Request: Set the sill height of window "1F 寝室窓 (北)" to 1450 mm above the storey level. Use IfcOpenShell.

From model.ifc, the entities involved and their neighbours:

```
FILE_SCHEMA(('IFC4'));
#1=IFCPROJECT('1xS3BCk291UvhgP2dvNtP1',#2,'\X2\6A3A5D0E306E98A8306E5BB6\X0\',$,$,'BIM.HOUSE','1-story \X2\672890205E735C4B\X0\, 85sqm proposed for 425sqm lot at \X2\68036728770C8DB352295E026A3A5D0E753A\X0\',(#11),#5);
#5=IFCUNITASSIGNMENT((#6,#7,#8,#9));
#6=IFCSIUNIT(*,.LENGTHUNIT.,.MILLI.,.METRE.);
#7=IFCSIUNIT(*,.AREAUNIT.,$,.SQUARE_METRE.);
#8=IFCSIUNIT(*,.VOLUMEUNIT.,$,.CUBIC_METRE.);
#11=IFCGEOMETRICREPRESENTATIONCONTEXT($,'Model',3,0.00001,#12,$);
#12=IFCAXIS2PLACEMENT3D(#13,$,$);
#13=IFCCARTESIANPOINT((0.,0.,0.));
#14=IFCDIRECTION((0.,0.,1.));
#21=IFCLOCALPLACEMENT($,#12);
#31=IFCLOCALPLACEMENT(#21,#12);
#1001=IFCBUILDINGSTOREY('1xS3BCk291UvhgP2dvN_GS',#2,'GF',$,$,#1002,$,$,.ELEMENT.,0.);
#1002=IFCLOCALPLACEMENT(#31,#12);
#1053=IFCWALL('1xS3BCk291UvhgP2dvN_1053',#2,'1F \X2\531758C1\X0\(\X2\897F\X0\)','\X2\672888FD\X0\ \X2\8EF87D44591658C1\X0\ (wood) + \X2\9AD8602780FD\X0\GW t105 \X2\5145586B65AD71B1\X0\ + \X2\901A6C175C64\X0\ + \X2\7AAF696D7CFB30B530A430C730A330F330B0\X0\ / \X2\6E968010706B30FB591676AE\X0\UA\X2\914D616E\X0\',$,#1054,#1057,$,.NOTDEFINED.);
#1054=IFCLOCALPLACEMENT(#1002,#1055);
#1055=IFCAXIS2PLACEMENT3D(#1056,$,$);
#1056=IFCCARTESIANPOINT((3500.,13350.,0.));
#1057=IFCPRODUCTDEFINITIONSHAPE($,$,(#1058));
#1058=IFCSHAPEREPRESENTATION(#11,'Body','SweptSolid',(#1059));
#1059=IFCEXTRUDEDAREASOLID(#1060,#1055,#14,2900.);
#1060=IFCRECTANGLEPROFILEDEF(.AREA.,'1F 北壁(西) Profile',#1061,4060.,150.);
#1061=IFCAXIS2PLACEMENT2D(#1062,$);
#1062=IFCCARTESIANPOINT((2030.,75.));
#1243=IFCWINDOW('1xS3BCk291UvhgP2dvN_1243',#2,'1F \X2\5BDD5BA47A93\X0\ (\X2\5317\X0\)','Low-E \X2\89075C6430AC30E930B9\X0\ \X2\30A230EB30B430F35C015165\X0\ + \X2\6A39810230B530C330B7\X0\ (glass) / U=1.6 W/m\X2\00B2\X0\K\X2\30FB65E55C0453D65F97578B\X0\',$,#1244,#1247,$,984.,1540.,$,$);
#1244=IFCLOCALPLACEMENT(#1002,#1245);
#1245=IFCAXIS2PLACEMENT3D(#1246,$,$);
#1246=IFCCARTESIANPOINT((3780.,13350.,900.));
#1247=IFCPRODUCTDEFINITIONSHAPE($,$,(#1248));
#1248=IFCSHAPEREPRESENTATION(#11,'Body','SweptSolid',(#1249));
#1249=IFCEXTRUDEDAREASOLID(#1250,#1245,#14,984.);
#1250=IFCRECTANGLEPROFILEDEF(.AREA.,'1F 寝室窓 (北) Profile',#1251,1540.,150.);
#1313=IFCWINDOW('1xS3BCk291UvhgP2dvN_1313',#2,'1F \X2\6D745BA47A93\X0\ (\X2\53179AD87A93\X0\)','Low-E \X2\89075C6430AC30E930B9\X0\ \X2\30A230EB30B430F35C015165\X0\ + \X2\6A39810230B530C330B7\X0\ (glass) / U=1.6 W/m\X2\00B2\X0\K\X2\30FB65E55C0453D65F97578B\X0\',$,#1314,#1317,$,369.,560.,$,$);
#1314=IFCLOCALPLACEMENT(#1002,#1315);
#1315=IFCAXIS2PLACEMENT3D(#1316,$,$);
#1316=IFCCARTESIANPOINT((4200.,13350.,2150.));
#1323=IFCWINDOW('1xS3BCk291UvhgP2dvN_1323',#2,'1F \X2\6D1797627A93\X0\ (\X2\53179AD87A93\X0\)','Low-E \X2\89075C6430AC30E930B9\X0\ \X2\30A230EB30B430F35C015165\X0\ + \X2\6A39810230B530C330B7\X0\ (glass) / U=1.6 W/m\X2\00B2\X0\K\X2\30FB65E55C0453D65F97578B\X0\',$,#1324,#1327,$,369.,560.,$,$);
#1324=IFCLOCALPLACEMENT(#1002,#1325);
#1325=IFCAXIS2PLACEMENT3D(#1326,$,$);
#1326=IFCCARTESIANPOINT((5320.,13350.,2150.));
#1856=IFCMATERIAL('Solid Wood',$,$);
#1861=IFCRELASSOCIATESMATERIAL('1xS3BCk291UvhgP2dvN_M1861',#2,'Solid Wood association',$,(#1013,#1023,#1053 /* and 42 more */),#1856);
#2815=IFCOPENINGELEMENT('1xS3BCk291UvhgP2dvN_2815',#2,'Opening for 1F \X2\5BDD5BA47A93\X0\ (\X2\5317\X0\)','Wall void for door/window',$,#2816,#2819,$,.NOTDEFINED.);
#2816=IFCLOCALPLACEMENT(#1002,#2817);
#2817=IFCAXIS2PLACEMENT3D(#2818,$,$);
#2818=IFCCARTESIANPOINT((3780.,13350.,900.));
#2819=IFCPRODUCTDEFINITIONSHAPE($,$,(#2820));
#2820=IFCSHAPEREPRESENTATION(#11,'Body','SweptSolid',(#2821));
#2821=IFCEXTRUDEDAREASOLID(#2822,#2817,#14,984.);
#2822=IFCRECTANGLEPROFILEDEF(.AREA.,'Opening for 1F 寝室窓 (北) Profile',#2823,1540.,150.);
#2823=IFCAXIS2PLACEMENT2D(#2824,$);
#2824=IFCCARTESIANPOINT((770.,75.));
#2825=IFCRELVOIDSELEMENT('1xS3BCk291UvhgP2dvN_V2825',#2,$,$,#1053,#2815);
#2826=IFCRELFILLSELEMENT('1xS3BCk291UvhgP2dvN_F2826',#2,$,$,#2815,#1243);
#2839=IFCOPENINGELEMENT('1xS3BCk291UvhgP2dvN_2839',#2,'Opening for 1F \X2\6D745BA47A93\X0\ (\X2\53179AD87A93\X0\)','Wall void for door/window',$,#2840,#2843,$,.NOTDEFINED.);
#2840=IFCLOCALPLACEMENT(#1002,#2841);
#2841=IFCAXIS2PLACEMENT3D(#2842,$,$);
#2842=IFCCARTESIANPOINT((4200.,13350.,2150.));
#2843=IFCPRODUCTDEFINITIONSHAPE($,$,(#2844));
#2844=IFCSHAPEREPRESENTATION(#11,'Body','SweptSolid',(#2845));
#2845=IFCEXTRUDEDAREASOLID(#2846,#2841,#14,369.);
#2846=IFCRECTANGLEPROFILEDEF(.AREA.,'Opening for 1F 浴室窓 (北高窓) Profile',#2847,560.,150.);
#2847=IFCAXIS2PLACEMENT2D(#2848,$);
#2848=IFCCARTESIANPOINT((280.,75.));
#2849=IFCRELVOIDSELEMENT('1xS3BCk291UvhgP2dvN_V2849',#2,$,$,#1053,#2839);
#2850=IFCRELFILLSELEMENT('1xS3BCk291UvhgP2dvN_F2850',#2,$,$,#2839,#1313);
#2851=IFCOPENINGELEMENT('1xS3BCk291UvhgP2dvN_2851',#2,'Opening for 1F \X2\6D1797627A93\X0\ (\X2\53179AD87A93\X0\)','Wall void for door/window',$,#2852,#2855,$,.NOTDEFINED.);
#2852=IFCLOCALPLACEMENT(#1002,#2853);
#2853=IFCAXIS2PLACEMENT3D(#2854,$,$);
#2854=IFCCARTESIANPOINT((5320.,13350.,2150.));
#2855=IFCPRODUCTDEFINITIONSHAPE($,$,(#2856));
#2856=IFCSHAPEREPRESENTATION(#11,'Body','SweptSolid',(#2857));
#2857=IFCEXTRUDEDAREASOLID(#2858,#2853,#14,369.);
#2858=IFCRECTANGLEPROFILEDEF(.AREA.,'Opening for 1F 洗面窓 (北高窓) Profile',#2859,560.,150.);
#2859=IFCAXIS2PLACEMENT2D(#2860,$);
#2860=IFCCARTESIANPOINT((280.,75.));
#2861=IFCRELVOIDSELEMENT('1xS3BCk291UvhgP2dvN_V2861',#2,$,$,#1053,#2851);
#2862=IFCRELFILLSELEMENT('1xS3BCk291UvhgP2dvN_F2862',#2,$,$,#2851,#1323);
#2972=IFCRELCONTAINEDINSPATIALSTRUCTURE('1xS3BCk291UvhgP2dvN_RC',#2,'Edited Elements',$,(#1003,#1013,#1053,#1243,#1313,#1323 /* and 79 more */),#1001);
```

```python
import numpy as np
import ifcopenshell
import ifcopenshell.api.geometry
import ifcopenshell.geom
import ifcopenshell.util.element
import ifcopenshell.util.placement
import ifcopenshell.util.shape
import ifcopenshell.util.unit

model = ifcopenshell.open("model.ifc")
unit_scale = ifcopenshell.util.unit.calculate_unit_scale(model)

window = model.by_guid("1xS3BCk291UvhgP2dvN_1243")
opening = window.FillsVoids[0].RelatingOpeningElement
storey = ifcopenshell.util.element.get_container(window, ifc_class="IfcBuildingStorey")
level = ifcopenshell.util.placement.get_local_placement(storey.ObjectPlacement)[2, 3]

# The opening's origin need not be at the sill, so measure its lowest point.
shape = ifcopenshell.geom.create_shape(ifcopenshell.geom.settings(), opening)
bottom = ifcopenshell.util.shape.get_shape_bottom_elevation(shape, shape.geometry) / unit_scale
dz = level + 1450.0 - bottom

shift = np.array([0.0, 0.0, dz])
# The window is not placed relative to its opening, so move both.
for product in (opening, window):
    matrix = ifcopenshell.util.placement.get_local_placement(product.ObjectPlacement)
    matrix[:3, 3] += shift
    ifcopenshell.api.geometry.edit_object_placement(model, product=product, matrix=matrix, is_si=False)

print(f"moved by {dz * unit_scale:+.3f} m")

model.write("model_updated.ifc")
```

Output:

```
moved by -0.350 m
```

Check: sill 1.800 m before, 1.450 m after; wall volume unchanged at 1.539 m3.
